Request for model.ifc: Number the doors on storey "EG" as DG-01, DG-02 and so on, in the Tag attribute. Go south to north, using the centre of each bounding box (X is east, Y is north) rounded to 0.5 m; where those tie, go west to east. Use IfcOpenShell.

First a look at what the model holds.

```python
import ifcopenshell
import ifcopenshell.util.element
import ifcopenshell.util.placement

model = ifcopenshell.open("model.ifc")
print(model.schema)
storey = next(s for s in model.by_type("IfcBuildingStorey") if s.Name == "EG")
doors = [e for e in ifcopenshell.util.element.get_decomposition(storey) if e.is_a("IfcDoor")]
for e in sorted(doors, key=lambda e: e.id()):
    origin = ifcopenshell.util.placement.get_local_placement(e.ObjectPlacement)[:3, 3]
    print(e.id(), e.Tag, e.Name, origin.round(2) + 0.0, sep=" | ")
```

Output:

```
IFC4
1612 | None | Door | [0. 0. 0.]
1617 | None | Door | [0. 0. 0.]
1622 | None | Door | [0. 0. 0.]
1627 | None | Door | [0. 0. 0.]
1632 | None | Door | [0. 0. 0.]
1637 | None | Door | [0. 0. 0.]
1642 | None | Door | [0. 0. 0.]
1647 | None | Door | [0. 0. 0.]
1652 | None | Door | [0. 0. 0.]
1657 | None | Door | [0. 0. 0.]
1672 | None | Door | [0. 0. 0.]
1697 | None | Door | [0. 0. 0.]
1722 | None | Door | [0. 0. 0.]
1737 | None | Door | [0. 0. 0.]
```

```python
import ifcopenshell
import ifcopenshell.geom
import ifcopenshell.util.element
import ifcopenshell.util.shape

model = ifcopenshell.open("model.ifc")
settings = ifcopenshell.geom.settings()
settings.set("use-world-coords", True)


def centre(element):
    shape = ifcopenshell.geom.create_shape(settings, element)
    return ifcopenshell.util.shape.get_bbox_centroid(shape.geometry)


storey = next(s for s in model.by_type("IfcBuildingStorey") if s.Name == "EG")
doors = [e for e in ifcopenshell.util.element.get_decomposition(storey) if e.is_a("IfcDoor")]

# Insertion points can sit at a corner or the storey origin, so sort by the geometry (in metres).
centres = {e: centre(e) for e in doors}
doors.sort(key=lambda e: (round(centres[e][1] / 0.5), centres[e][0]))

for i, e in enumerate(doors, start=1):
    number = f"DG-{i:02d}"
    e.Tag = number
    print(e.id(), number)

model.write("model_v2.ifc")
```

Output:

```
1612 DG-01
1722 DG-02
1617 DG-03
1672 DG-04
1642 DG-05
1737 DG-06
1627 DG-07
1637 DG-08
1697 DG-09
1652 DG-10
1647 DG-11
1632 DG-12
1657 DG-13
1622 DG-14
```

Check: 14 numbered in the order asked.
